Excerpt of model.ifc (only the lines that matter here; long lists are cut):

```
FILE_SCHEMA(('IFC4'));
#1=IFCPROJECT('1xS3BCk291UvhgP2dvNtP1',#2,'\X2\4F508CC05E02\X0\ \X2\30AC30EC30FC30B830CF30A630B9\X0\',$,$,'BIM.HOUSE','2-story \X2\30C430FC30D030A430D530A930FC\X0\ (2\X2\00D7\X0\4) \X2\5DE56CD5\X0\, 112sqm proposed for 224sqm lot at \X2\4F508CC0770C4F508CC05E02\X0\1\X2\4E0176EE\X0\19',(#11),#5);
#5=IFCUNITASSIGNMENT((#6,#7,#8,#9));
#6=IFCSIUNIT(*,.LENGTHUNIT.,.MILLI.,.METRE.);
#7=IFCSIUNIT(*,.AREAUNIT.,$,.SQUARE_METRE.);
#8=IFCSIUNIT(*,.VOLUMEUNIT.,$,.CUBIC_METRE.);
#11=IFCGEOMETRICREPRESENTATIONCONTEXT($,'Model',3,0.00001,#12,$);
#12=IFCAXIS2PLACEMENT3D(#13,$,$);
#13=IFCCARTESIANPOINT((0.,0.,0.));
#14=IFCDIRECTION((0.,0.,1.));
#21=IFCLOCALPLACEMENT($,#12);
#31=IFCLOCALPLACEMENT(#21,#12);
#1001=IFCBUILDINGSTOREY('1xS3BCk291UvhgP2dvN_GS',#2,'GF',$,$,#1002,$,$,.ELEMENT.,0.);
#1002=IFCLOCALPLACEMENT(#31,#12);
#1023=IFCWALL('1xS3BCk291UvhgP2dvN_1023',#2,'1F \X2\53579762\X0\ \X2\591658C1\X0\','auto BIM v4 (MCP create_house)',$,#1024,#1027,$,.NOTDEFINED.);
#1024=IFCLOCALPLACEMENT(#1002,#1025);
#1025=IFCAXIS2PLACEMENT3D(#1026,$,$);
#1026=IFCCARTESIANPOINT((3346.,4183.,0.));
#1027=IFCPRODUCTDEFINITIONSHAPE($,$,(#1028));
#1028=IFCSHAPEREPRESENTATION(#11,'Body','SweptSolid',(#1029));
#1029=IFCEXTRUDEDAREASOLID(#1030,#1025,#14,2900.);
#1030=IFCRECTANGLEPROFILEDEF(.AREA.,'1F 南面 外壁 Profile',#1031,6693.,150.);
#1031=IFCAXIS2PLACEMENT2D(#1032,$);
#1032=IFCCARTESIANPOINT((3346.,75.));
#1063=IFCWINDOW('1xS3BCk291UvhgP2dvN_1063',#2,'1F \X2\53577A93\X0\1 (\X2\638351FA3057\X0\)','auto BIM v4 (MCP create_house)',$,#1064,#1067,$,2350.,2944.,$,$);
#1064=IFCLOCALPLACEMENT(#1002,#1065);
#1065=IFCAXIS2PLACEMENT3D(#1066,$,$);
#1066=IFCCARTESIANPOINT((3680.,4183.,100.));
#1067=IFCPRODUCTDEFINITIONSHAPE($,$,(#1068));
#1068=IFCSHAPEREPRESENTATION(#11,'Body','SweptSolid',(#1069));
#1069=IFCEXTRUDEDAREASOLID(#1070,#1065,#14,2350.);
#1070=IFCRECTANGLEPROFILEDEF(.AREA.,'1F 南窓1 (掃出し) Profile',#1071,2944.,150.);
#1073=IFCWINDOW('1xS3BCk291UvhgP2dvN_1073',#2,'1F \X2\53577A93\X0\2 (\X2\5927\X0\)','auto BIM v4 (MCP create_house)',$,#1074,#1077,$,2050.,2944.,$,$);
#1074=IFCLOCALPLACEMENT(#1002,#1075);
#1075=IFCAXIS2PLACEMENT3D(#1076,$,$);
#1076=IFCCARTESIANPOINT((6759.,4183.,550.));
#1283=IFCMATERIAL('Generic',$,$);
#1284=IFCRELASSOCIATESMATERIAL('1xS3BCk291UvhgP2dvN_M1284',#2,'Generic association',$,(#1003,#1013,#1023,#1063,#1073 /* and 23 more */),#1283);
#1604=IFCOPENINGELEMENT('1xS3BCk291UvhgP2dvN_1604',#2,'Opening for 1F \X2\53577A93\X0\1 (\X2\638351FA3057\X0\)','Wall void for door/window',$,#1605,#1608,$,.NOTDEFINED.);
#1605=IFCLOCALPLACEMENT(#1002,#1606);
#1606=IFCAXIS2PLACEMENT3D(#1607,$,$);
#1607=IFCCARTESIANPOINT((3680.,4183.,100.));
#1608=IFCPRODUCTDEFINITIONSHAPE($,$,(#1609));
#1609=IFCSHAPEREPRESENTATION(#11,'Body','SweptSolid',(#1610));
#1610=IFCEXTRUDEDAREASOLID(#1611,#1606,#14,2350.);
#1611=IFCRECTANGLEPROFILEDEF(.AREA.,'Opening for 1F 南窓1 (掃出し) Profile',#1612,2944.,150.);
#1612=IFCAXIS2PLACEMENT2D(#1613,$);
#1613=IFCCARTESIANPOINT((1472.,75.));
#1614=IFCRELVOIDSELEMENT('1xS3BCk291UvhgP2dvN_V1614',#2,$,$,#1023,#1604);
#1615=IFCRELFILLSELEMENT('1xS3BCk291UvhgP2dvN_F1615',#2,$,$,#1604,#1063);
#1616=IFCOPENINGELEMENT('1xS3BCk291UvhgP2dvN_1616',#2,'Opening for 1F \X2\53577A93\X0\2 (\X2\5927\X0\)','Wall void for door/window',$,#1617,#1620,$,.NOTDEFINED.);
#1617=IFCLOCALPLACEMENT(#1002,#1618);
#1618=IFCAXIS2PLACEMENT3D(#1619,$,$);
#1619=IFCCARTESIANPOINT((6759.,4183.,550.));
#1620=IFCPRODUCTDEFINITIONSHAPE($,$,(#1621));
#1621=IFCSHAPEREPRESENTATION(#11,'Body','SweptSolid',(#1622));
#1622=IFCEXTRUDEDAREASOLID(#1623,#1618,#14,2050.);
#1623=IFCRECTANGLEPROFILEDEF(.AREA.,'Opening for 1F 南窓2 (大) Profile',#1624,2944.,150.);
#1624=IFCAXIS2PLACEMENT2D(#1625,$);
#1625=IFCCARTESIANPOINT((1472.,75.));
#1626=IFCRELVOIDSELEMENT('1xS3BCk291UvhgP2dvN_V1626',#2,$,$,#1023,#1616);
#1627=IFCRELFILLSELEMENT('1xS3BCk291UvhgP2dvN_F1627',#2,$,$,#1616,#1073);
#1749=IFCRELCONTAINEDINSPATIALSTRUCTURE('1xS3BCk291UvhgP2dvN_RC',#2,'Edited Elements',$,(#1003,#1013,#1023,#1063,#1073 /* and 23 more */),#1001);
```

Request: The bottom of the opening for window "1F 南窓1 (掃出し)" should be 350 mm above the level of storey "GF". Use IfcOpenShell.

```python
import numpy as np
import ifcopenshell
import ifcopenshell.api.geometry
import ifcopenshell.geom
import ifcopenshell.util.element
import ifcopenshell.util.placement
import ifcopenshell.util.shape
import ifcopenshell.util.unit

model = ifcopenshell.open("model.ifc")
unit_scale = ifcopenshell.util.unit.calculate_unit_scale(model)

window = model.by_guid("1xS3BCk291UvhgP2dvN_1063")
opening = window.FillsVoids[0].RelatingOpeningElement
storey = ifcopenshell.util.element.get_container(window, ifc_class="IfcBuildingStorey")
level = ifcopenshell.util.placement.get_local_placement(storey.ObjectPlacement)[2, 3]

# The opening's origin need not be at the sill, so measure its lowest point.
shape = ifcopenshell.geom.create_shape(ifcopenshell.geom.settings(), opening)
bottom = ifcopenshell.util.shape.get_shape_bottom_elevation(shape, shape.geometry) / unit_scale
dz = level + 0.35 / unit_scale - bottom

shift = np.array([0.0, 0.0, dz])
# The window is not placed relative to its opening, so move both.
for product in (opening, window):
    matrix = ifcopenshell.util.placement.get_local_placement(product.ObjectPlacement)
    matrix[:3, 3] += shift
    ifcopenshell.api.geometry.edit_object_placement(model, product=product, matrix=matrix, is_si=False)

print(f"moved by {dz * unit_scale:+.3f} m")

model.write("model_updated.ifc")
```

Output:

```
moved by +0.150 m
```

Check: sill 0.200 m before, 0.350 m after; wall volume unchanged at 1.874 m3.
